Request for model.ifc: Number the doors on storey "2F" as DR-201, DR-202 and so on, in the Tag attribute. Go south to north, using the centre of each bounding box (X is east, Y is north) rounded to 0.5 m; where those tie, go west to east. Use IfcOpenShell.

First a look at what the model holds.

```python
import ifcopenshell
import ifcopenshell.util.element
import ifcopenshell.util.placement

model = ifcopenshell.open("model.ifc")
print(model.schema)
storey = next(s for s in model.by_type("IfcBuildingStorey") if s.Name == "2F")
doors = [e for e in ifcopenshell.util.element.get_decomposition(storey) if e.is_a("IfcDoor")]
for e in sorted(doors, key=lambda e: e.id()):
    origin = ifcopenshell.util.placement.get_local_placement(e.ObjectPlacement)[:3, 3]
    print(e.id(), e.Tag, e.Name, origin.round(2) + 0.0, sep=" | ")
```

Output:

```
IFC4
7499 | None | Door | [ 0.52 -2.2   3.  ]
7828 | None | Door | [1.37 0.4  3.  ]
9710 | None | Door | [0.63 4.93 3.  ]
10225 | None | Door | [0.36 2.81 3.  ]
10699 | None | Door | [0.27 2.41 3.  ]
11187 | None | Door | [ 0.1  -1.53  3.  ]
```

```python
import ifcopenshell
import ifcopenshell.geom
import ifcopenshell.util.element
import ifcopenshell.util.shape

model = ifcopenshell.open("model.ifc")
settings = ifcopenshell.geom.settings()
settings.set("use-world-coords", True)


def centre(element):
    shape = ifcopenshell.geom.create_shape(settings, element)
    return ifcopenshell.util.shape.get_bbox_centroid(shape.geometry)


storey = next(s for s in model.by_type("IfcBuildingStorey") if s.Name == "2F")
doors = [e for e in ifcopenshell.util.element.get_decomposition(storey) if e.is_a("IfcDoor")]

# Insertion points can sit at a corner or the storey origin, so sort by the geometry (in metres).
centres = {e: centre(e) for e in doors}
doors.sort(key=lambda e: (round(centres[e][1] / 0.5), centres[e][0]))

for i, e in enumerate(doors, start=1):
    number = f"DR-2{i:02d}"
    e.Tag = number
    print(e.id(), number)

model.write("model_rev.ifc")
```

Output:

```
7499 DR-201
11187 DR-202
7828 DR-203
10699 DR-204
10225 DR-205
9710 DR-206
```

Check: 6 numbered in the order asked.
